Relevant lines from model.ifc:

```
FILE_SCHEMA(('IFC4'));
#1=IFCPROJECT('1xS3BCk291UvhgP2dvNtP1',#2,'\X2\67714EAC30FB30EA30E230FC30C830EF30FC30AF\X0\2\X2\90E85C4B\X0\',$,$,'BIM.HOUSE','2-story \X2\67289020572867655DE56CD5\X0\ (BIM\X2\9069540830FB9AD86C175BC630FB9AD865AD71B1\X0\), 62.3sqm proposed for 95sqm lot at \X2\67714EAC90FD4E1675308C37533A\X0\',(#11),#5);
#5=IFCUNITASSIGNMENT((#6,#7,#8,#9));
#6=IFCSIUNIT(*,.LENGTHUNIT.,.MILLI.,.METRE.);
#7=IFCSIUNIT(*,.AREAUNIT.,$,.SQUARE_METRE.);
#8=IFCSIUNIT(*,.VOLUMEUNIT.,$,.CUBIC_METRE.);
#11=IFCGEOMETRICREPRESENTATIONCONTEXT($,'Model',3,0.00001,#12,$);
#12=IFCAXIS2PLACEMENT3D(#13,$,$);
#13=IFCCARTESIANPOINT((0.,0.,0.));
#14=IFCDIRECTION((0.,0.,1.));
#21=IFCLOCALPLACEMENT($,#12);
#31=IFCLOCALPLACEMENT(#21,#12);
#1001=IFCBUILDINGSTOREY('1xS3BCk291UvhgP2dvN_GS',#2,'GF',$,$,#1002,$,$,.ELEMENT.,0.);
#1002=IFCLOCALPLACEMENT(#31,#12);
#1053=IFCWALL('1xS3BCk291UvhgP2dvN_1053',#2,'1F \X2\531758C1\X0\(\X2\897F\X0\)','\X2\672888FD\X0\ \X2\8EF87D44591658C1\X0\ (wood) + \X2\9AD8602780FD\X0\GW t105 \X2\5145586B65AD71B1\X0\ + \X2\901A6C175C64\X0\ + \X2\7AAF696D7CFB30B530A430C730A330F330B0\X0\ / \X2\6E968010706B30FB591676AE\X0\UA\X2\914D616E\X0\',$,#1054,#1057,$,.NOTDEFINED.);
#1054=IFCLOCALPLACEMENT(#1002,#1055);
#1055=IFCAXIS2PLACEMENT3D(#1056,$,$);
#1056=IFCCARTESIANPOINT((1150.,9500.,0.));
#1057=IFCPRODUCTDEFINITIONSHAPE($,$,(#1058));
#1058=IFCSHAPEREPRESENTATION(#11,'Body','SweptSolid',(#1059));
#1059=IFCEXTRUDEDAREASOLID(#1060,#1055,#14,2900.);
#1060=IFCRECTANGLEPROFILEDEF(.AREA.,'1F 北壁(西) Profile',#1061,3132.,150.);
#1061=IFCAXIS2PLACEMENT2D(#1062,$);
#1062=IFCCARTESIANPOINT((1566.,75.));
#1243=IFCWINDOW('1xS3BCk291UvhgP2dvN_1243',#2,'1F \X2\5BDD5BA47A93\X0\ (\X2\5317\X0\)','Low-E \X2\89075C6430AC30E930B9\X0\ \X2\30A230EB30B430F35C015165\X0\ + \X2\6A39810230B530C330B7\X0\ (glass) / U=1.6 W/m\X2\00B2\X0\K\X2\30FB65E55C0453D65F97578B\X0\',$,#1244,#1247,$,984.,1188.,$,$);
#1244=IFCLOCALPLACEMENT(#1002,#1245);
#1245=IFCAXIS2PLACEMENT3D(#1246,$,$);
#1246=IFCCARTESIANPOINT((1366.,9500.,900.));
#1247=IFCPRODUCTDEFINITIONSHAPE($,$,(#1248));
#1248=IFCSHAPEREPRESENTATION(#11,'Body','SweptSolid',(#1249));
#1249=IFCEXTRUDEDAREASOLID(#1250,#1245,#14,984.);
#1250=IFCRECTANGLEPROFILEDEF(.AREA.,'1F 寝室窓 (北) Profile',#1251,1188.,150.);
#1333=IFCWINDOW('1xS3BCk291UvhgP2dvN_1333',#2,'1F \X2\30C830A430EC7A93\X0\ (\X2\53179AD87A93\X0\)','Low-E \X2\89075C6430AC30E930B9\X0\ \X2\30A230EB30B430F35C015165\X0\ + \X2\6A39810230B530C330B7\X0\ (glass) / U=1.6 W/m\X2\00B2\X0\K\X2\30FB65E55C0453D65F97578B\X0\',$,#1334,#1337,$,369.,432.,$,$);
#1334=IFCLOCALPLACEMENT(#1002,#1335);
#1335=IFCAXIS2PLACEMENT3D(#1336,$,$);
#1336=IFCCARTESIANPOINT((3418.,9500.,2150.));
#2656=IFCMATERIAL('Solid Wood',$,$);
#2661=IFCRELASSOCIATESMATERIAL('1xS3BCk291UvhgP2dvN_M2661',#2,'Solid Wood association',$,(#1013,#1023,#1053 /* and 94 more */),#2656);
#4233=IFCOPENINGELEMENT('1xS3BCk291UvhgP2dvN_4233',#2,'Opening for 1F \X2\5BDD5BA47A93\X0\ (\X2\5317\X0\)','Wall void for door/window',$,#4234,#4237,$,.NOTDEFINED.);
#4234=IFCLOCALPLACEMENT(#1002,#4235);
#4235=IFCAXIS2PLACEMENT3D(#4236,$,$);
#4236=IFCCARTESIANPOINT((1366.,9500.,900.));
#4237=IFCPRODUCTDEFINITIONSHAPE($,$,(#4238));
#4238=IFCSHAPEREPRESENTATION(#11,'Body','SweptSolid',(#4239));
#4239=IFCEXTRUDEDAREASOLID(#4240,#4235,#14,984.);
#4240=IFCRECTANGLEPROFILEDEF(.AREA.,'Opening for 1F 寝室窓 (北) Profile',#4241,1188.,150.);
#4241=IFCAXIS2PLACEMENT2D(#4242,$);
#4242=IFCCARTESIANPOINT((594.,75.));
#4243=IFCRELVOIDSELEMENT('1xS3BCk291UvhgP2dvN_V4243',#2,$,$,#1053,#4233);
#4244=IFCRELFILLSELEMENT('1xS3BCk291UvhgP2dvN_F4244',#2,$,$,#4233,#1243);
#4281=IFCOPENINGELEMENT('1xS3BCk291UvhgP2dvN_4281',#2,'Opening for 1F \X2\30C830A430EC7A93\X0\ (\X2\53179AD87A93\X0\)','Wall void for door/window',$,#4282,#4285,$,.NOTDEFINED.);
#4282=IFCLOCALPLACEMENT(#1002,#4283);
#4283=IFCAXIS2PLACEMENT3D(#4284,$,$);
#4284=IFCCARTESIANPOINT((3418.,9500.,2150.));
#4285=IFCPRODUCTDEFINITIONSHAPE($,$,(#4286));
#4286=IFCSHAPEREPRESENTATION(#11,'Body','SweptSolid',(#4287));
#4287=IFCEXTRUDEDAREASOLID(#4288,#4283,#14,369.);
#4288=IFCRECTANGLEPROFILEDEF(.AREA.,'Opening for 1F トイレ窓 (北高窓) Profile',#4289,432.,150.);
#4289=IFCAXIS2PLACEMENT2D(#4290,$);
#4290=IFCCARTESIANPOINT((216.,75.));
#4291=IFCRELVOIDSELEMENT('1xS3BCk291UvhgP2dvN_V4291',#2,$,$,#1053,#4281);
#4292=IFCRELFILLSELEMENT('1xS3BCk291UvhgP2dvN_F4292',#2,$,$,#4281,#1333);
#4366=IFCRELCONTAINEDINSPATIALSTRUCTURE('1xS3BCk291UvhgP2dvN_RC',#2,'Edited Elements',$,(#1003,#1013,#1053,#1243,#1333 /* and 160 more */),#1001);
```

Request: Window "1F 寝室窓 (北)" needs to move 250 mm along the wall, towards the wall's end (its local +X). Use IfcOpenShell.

```python
import ifcopenshell
import ifcopenshell.api.geometry
import ifcopenshell.util.placement

model = ifcopenshell.open("model.ifc")

window = model.by_id(1243)
opening = window.FillsVoids[0].RelatingOpeningElement
wall = opening.VoidsElements[0].RelatingBuildingElement

wall_matrix = ifcopenshell.util.placement.get_local_placement(wall.ObjectPlacement)
shift = wall_matrix[:3, 0] * 250.0
before = ifcopenshell.util.placement.get_local_placement(window.ObjectPlacement)[:3, 3].copy()

# The window is not placed relative to its opening, so move both.
for product in (opening, window):
    matrix = ifcopenshell.util.placement.get_local_placement(product.ObjectPlacement)
    matrix[:3, 3] += shift
    ifcopenshell.api.geometry.edit_object_placement(model, product=product, matrix=matrix, is_si=False)

after = ifcopenshell.util.placement.get_local_placement(window.ObjectPlacement)[:3, 3]
print("window moved by", (after - before).round(3) + 0.0)

model.write("model_rev.ifc")
```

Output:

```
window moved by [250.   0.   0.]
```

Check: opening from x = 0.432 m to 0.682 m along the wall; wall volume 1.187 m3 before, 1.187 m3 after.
